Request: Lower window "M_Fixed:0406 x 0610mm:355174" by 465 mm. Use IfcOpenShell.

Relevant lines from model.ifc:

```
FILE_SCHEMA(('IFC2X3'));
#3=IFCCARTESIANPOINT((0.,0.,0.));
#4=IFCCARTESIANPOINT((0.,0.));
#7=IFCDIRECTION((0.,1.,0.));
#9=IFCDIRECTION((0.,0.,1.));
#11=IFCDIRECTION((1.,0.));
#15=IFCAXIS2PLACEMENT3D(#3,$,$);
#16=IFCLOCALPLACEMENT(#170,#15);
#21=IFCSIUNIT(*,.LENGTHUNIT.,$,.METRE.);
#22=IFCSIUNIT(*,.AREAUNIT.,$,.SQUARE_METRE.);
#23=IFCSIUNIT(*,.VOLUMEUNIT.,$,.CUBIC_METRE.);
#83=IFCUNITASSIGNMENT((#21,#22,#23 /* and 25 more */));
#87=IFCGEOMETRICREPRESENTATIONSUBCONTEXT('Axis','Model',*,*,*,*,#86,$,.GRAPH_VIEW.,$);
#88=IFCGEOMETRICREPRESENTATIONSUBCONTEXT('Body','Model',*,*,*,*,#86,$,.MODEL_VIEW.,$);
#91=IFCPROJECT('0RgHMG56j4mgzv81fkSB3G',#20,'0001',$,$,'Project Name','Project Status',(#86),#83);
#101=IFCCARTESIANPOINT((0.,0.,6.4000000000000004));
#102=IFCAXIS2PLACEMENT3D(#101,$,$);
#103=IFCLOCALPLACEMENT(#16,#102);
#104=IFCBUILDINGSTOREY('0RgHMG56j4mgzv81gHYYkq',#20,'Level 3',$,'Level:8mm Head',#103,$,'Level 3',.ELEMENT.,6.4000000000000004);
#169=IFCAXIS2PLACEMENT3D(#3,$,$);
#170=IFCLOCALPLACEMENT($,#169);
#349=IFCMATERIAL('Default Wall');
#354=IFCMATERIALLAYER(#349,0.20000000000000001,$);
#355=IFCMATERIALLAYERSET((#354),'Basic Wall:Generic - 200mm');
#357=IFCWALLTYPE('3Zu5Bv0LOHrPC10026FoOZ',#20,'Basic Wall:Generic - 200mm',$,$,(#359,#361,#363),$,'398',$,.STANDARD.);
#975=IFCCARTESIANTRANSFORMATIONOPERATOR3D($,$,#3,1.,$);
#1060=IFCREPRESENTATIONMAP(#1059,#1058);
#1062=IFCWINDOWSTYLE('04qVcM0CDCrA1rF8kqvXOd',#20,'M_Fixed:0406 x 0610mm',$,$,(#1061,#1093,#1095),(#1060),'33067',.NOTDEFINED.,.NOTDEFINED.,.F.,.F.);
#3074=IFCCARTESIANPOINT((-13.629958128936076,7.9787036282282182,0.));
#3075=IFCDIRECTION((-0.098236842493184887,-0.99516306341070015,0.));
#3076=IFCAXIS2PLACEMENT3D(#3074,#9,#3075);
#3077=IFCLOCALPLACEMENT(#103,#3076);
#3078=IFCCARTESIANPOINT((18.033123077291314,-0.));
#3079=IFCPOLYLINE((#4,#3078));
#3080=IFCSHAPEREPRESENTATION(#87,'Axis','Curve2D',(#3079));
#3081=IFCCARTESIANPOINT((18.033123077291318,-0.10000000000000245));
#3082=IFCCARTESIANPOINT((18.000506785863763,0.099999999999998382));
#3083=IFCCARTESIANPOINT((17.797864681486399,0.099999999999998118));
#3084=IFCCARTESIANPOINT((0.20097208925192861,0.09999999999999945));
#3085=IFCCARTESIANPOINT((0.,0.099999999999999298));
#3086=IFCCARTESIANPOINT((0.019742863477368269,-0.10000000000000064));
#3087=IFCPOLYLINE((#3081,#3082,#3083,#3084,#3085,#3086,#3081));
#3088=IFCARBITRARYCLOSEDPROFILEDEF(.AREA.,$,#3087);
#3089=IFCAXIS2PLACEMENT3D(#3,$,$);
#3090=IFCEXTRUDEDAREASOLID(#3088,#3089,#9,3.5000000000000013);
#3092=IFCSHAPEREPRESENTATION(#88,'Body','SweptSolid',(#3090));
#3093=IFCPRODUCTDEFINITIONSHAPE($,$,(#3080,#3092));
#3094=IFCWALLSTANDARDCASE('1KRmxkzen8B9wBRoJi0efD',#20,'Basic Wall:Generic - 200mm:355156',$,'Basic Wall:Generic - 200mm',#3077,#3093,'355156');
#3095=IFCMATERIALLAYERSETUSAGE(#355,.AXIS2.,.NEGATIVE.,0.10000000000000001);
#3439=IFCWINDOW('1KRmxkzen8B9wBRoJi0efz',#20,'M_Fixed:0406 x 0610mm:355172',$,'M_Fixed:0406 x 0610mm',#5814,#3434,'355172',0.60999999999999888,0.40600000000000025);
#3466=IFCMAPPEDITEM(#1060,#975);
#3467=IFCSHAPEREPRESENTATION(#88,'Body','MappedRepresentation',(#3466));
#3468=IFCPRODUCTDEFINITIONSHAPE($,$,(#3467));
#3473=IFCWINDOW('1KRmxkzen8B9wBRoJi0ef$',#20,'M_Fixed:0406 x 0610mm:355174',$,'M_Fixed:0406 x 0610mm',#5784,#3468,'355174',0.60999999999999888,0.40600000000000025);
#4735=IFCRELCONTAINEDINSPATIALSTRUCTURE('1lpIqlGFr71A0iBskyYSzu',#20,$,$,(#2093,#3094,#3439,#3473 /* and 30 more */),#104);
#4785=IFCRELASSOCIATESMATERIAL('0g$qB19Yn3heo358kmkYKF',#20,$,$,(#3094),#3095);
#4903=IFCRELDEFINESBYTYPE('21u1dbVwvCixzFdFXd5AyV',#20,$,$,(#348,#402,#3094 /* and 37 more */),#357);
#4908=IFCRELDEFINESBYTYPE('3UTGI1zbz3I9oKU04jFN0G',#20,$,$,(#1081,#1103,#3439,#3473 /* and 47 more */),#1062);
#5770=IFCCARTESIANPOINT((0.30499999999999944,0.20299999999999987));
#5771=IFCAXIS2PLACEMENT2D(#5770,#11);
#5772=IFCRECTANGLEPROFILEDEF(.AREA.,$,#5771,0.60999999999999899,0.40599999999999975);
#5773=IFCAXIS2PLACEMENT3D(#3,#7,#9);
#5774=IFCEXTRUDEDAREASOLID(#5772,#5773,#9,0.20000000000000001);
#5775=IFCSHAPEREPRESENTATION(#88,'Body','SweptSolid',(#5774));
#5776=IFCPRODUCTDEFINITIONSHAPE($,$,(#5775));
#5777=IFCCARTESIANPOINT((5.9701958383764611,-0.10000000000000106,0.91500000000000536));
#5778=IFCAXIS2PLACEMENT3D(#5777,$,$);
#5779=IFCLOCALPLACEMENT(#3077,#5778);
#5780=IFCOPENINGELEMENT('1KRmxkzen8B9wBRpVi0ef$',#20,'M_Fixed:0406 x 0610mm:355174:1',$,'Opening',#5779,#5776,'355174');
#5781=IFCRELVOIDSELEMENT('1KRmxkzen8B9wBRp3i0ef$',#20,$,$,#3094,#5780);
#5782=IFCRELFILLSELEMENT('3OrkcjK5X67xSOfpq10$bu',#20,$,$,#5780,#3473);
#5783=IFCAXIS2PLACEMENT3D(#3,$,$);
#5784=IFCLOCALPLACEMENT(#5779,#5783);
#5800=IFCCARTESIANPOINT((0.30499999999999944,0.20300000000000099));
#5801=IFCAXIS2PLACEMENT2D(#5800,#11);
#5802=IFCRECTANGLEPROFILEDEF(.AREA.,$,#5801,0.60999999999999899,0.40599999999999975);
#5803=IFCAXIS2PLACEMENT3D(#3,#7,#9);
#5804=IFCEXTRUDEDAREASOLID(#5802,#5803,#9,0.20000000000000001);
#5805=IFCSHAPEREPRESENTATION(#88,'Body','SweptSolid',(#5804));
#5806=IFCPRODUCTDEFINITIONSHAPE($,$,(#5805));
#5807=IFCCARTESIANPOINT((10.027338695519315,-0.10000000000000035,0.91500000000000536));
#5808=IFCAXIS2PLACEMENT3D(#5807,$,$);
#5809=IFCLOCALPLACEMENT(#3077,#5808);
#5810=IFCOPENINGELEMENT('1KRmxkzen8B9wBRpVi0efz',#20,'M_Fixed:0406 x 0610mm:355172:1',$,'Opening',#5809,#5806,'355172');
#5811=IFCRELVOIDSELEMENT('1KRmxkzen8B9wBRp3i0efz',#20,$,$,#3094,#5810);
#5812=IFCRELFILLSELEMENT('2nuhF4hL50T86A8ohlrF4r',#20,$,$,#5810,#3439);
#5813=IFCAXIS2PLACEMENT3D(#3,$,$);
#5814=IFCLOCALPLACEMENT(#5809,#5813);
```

```python
import numpy as np
import ifcopenshell
import ifcopenshell.api.geometry
import ifcopenshell.util.placement
import ifcopenshell.util.unit

model = ifcopenshell.open("model.ifc")
unit_scale = ifcopenshell.util.unit.calculate_unit_scale(model)

window = model.by_id(3473)
opening = window.FillsVoids[0].RelatingOpeningElement
dz = -0.465 / unit_scale

shift = np.array([0.0, 0.0, dz])
# The window is placed relative to its opening, so it follows when the opening moves.
matrix = ifcopenshell.util.placement.get_local_placement(opening.ObjectPlacement)
matrix[:3, 3] += shift
ifcopenshell.api.geometry.edit_object_placement(
    model, product=opening, matrix=matrix, is_si=False, should_transform_children=True
)

print(f"moved by {dz * unit_scale:+.3f} m")

model.write("model_updated.ifc")
```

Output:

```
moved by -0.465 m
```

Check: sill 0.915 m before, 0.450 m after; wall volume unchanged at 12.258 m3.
